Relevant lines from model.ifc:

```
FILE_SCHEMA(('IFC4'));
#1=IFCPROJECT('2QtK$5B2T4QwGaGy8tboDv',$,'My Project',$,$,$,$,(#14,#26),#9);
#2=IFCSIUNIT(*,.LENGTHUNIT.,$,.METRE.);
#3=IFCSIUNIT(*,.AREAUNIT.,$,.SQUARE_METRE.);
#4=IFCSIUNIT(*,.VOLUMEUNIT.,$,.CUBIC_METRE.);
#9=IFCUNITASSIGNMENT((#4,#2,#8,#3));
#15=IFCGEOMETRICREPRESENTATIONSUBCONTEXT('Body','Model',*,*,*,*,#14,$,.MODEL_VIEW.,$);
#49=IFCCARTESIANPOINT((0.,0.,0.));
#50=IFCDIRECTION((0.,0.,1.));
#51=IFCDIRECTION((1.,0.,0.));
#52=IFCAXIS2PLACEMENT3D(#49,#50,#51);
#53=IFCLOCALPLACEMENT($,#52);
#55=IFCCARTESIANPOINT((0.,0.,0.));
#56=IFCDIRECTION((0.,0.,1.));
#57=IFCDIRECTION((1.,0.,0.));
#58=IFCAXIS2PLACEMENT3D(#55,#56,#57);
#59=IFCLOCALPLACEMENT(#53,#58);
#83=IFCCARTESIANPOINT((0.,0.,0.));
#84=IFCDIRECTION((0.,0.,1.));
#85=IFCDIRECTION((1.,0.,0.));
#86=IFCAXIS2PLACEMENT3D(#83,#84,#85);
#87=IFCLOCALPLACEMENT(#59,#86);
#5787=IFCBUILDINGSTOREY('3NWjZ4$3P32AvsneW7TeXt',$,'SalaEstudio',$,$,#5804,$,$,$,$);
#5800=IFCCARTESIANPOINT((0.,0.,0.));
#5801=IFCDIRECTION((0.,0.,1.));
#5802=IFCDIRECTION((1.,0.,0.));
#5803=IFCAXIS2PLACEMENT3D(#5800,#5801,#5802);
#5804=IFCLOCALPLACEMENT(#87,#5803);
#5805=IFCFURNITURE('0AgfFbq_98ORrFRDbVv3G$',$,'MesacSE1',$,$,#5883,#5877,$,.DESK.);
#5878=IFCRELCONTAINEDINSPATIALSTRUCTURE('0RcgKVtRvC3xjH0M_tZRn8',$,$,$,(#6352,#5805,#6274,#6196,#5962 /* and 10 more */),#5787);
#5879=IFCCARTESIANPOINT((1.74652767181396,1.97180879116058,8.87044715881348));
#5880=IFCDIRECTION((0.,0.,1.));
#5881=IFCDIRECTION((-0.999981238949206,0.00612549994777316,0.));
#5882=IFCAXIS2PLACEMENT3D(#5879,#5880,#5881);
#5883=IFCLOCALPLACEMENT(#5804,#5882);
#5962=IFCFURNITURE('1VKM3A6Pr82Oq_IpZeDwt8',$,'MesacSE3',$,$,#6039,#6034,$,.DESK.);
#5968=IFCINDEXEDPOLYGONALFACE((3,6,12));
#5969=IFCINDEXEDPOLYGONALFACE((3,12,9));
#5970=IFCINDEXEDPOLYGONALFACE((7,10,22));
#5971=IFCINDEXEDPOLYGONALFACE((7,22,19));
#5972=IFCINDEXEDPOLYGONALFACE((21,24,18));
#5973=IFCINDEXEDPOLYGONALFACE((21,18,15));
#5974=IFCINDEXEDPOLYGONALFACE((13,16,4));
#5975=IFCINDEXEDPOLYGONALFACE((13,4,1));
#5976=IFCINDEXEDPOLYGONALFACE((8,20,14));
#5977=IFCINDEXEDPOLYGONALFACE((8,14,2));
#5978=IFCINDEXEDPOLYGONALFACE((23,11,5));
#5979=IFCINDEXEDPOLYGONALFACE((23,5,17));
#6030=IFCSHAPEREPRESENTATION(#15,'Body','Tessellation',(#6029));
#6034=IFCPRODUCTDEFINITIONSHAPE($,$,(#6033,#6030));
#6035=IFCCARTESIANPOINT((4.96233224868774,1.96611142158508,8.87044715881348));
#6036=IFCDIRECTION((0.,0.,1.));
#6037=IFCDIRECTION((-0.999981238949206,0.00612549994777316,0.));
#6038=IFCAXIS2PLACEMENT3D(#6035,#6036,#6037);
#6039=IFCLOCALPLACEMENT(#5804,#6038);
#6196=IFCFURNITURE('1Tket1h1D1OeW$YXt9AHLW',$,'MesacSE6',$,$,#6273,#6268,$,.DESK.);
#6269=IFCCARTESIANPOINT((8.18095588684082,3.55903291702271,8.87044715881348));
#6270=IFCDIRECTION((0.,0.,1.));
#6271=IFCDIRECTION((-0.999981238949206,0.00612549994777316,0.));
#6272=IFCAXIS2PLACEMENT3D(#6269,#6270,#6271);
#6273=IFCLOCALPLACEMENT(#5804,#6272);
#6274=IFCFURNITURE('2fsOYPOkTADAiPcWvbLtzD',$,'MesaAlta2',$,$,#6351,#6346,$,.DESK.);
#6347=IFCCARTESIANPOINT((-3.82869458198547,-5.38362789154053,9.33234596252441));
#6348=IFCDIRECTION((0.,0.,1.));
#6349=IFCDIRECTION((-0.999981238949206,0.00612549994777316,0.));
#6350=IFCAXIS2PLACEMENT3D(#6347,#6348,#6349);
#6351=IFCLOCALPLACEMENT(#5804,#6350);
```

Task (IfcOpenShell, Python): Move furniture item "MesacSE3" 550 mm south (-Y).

```python
import ifcopenshell
import ifcopenshell.api.geometry
import ifcopenshell.util.placement
import ifcopenshell.util.unit

model = ifcopenshell.open("model.ifc")
unit_scale = ifcopenshell.util.unit.calculate_unit_scale(model)

item = model.by_guid("1VKM3A6Pr82Oq_IpZeDwt8")
matrix = ifcopenshell.util.placement.get_local_placement(item.ObjectPlacement)
matrix[1, 3] -= 0.55 / unit_scale
ifcopenshell.api.geometry.edit_object_placement(model, product=item, matrix=matrix, is_si=False)

print(ifcopenshell.util.placement.get_local_placement(item.ObjectPlacement).round(3) + 0.0)

model.write("model_rev.ifc")
```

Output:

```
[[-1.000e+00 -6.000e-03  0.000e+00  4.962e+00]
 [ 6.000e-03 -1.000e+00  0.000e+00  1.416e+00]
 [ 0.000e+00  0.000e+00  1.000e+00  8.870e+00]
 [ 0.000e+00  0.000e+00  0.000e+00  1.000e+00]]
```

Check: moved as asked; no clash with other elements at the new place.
